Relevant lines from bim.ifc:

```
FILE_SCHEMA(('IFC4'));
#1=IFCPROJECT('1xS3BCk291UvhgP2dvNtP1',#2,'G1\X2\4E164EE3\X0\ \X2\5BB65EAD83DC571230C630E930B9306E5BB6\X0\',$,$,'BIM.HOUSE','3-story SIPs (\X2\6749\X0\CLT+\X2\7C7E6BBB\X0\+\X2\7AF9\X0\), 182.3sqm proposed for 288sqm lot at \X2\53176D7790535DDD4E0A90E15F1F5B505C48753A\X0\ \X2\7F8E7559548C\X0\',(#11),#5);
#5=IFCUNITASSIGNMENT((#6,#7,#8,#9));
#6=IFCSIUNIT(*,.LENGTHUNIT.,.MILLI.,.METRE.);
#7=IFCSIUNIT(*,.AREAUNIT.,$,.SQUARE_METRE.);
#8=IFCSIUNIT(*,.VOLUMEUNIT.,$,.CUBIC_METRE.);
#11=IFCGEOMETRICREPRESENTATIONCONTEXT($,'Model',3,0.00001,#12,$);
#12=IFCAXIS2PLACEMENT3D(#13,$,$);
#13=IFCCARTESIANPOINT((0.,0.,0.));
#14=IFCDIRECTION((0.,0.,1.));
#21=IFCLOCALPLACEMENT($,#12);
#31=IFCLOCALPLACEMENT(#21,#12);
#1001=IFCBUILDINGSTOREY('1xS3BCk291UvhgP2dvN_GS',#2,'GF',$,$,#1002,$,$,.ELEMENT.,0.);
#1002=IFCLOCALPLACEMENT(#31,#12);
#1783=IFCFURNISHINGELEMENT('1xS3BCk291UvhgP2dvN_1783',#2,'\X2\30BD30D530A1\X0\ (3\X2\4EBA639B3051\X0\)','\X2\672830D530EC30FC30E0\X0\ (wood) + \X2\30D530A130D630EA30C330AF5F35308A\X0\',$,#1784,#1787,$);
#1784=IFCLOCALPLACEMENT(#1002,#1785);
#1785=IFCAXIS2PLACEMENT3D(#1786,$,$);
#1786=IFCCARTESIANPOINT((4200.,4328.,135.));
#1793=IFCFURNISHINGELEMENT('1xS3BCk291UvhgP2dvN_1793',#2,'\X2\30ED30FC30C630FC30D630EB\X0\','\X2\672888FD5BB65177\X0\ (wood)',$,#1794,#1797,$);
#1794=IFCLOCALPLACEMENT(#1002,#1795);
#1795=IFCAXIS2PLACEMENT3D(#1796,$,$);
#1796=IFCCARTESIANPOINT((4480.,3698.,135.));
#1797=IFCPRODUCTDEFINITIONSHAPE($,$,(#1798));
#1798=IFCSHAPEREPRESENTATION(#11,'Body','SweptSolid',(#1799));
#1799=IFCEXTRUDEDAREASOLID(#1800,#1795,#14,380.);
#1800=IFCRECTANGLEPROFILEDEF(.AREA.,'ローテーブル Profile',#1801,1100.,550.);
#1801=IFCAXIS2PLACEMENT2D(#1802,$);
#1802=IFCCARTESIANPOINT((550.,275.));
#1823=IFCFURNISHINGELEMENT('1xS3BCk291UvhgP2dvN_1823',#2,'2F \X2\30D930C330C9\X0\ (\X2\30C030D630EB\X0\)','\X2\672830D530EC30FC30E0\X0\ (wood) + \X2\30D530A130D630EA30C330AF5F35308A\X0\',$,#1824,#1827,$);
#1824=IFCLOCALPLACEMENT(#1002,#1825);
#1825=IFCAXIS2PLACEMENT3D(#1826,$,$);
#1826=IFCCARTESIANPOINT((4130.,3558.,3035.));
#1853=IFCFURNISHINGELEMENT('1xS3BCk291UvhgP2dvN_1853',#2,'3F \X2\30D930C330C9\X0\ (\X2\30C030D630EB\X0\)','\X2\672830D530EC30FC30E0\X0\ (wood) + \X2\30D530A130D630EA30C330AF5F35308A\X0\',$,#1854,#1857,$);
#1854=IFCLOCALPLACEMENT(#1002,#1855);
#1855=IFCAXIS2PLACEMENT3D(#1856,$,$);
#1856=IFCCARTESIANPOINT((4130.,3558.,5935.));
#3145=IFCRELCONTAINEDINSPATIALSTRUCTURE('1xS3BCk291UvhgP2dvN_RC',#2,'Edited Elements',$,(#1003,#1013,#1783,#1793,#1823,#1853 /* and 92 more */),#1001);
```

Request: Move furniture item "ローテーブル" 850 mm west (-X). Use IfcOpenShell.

```python
import ifcopenshell
import ifcopenshell.api.geometry
import ifcopenshell.util.placement
import ifcopenshell.util.unit

model = ifcopenshell.open("bim.ifc")
unit_scale = ifcopenshell.util.unit.calculate_unit_scale(model)

item = model.by_guid("1xS3BCk291UvhgP2dvN_1793")
matrix = ifcopenshell.util.placement.get_local_placement(item.ObjectPlacement)
matrix[0, 3] -= 0.85 / unit_scale
ifcopenshell.api.geometry.edit_object_placement(model, product=item, matrix=matrix, is_si=False)

print(ifcopenshell.util.placement.get_local_placement(item.ObjectPlacement).round(3) + 0.0)

model.write("bim_edited.ifc")
```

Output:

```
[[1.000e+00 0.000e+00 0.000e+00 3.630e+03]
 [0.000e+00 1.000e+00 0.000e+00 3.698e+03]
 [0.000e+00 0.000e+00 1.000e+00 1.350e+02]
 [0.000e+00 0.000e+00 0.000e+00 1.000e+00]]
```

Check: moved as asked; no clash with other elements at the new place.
